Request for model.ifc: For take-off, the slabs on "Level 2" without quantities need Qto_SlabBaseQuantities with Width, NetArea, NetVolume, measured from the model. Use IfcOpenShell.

First a look at what the model holds.

```python
import ifcopenshell
import ifcopenshell.util.element
import ifcopenshell.util.unit

model = ifcopenshell.open("model.ifc")
print(model.schema)
for unit_type in ("LENGTHUNIT", "AREAUNIT", "VOLUMEUNIT"):
    print(unit_type, ifcopenshell.util.unit.calculate_unit_scale(model, unit_type))
storey = next(s for s in model.by_type("IfcBuildingStorey") if s.Name == "Level 2")
slabs = [e for e in ifcopenshell.util.element.get_decomposition(storey) if e.is_a("IfcSlab")]
for e in sorted(slabs, key=lambda e: e.id()):
    print(e.id(), e.is_a(), e.Name, list(ifcopenshell.util.element.get_psets(e, qtos_only=True)), sep=" | ")
```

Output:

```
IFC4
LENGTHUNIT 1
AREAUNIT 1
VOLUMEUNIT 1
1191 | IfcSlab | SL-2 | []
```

```python
import ifcopenshell
import ifcopenshell.api.pset
import ifcopenshell.geom
import ifcopenshell.util.element
import ifcopenshell.util.shape
import ifcopenshell.util.unit

model = ifcopenshell.open("model.ifc")
unit_scale = ifcopenshell.util.unit.calculate_unit_scale(model)
area_scale = ifcopenshell.util.unit.calculate_unit_scale(model, "AREAUNIT")
volume_scale = ifcopenshell.util.unit.calculate_unit_scale(model, "VOLUMEUNIT")
settings = ifcopenshell.geom.settings()

storey = next(s for s in model.by_type("IfcBuildingStorey") if s.Name == "Level 2")
slabs = [e for e in ifcopenshell.util.element.get_decomposition(storey) if e.is_a("IfcSlab")]

for e in sorted(slabs, key=lambda e: e.id()):
    if ifcopenshell.util.element.get_psets(e, qtos_only=True, should_inherit=False):
        continue
    # Geometry comes back in metres, in the element's own axes.
    shape = ifcopenshell.geom.create_shape(settings, e)
    values = {
        "Width": ifcopenshell.util.shape.get_z(shape.geometry) / unit_scale,
        "NetArea": ifcopenshell.util.shape.get_footprint_area(shape.geometry) / area_scale,
        "NetVolume": ifcopenshell.util.shape.get_volume(shape.geometry) / volume_scale,
    }
    qto = ifcopenshell.api.pset.add_qto(model, product=e, name="Qto_SlabBaseQuantities")
    ifcopenshell.api.pset.edit_qto(model, qto=qto, properties=values)
    print(e.id(), {k: round(v, 3) for k, v in values.items()})

model.write("model_v2.ifc")
```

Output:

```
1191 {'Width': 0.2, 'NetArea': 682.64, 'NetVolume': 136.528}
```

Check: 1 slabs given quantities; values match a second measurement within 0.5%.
